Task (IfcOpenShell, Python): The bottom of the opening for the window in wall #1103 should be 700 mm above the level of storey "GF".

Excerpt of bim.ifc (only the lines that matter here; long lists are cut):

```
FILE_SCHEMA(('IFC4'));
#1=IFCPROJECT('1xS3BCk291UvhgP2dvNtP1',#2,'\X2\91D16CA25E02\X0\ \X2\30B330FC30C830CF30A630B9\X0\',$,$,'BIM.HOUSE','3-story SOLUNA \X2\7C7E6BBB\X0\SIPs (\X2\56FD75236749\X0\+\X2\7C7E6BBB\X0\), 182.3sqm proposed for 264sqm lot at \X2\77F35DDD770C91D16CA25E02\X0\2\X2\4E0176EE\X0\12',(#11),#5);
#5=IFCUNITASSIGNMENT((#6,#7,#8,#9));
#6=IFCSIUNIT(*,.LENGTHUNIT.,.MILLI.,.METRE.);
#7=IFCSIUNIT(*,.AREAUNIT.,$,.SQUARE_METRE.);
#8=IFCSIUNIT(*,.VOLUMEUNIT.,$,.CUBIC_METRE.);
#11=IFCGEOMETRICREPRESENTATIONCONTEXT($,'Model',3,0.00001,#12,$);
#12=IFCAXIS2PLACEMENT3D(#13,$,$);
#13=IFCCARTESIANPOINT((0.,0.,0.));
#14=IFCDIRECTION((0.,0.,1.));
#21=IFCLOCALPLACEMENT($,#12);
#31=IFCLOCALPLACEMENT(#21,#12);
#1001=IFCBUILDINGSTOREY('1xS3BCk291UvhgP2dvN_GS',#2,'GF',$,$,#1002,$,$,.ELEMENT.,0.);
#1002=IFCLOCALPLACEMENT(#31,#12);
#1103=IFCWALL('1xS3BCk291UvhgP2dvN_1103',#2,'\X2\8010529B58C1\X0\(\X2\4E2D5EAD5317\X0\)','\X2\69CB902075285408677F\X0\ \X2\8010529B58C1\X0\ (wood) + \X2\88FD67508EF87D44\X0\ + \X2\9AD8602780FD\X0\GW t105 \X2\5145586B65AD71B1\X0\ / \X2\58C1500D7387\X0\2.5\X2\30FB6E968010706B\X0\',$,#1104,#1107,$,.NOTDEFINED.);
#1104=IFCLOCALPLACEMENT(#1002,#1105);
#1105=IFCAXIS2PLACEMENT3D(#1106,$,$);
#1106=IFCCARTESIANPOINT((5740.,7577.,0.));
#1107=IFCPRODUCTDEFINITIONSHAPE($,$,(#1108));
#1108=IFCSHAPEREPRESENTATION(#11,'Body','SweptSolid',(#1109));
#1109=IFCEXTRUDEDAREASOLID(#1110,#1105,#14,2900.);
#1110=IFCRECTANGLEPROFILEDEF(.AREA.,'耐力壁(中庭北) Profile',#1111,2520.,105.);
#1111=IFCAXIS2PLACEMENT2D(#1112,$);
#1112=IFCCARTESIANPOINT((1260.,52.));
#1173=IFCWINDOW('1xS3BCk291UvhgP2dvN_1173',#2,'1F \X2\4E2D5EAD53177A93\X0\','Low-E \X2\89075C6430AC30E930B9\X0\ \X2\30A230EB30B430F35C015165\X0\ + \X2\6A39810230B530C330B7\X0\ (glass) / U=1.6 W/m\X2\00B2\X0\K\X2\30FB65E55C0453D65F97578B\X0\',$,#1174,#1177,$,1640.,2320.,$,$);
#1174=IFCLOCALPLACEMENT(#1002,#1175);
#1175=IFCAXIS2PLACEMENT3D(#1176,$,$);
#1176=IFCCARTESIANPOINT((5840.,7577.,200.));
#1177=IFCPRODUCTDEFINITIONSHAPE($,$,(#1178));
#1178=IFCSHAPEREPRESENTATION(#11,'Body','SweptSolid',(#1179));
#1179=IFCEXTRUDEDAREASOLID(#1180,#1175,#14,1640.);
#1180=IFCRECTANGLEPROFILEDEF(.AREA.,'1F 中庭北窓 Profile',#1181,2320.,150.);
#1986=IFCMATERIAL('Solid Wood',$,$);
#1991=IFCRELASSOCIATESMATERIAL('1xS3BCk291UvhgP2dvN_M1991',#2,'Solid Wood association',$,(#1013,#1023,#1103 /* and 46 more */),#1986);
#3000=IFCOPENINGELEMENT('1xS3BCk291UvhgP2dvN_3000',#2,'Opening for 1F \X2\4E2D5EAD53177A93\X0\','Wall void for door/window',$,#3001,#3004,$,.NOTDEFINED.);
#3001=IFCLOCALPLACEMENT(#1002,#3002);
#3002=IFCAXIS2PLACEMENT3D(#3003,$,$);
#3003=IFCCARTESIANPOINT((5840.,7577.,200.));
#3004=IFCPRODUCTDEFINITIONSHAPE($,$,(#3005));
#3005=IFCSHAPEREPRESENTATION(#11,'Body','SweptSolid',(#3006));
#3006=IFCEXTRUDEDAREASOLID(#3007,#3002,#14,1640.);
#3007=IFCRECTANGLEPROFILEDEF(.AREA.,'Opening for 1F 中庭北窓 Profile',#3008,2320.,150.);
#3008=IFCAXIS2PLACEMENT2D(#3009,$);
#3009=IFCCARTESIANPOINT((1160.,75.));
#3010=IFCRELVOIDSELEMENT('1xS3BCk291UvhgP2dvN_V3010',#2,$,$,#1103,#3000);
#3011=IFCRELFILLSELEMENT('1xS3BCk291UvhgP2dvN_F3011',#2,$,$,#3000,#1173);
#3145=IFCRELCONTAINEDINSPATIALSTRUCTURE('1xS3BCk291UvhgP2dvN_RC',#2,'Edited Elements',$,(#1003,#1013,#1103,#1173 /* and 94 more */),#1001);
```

```python
import numpy as np
import ifcopenshell
import ifcopenshell.api.geometry
import ifcopenshell.geom
import ifcopenshell.util.element
import ifcopenshell.util.placement
import ifcopenshell.util.shape
import ifcopenshell.util.unit

model = ifcopenshell.open("bim.ifc")
unit_scale = ifcopenshell.util.unit.calculate_unit_scale(model)

window = model.by_id(1173)
opening = window.FillsVoids[0].RelatingOpeningElement
storey = ifcopenshell.util.element.get_container(window, ifc_class="IfcBuildingStorey")
level = ifcopenshell.util.placement.get_local_placement(storey.ObjectPlacement)[2, 3]

# The opening's origin need not be at the sill, so measure its lowest point.
shape = ifcopenshell.geom.create_shape(ifcopenshell.geom.settings(), opening)
bottom = ifcopenshell.util.shape.get_shape_bottom_elevation(shape, shape.geometry) / unit_scale
dz = level + 700.0 - bottom

shift = np.array([0.0, 0.0, dz])
# The window is not placed relative to its opening, so move both.
for product in (opening, window):
    matrix = ifcopenshell.util.placement.get_local_placement(product.ObjectPlacement)
    matrix[:3, 3] += shift
    ifcopenshell.api.geometry.edit_object_placement(model, product=product, matrix=matrix, is_si=False)

print(f"moved by {dz * unit_scale:+.3f} m")

model.write("bim_updated.ifc")
```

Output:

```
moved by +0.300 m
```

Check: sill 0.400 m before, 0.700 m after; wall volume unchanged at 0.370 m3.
